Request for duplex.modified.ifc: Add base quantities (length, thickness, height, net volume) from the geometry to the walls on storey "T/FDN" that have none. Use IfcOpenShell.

First a look at what the model holds.

```python
import ifcopenshell
import ifcopenshell.util.element
import ifcopenshell.util.unit

model = ifcopenshell.open("duplex.modified.ifc")
print(model.schema)
for unit_type in ("LENGTHUNIT", "AREAUNIT", "VOLUMEUNIT"):
    print(unit_type, ifcopenshell.util.unit.calculate_unit_scale(model, unit_type))
storey = next(s for s in model.by_type("IfcBuildingStorey") if s.Name == "T/FDN")
walls = [e for e in ifcopenshell.util.element.get_decomposition(storey) if e.is_a("IfcWall")]
for e in sorted(walls, key=lambda e: e.id()):
    print(e.id(), e.is_a(), e.Name, list(ifcopenshell.util.element.get_psets(e, qtos_only=True)), sep=" | ")
```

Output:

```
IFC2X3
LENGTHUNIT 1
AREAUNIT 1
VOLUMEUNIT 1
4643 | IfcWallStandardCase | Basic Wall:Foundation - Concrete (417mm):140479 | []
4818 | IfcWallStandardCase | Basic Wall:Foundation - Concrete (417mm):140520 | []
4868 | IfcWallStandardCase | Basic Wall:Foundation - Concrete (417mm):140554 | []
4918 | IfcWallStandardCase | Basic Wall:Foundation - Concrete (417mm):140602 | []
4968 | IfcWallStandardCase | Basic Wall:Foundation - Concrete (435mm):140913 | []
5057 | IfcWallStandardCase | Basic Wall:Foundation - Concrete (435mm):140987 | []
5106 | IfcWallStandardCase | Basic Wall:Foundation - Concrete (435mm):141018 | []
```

```python
import ifcopenshell
import ifcopenshell.api.pset
import ifcopenshell.geom
import ifcopenshell.util.element
import ifcopenshell.util.shape
import ifcopenshell.util.unit

model = ifcopenshell.open("duplex.modified.ifc")
unit_scale = ifcopenshell.util.unit.calculate_unit_scale(model)
volume_scale = ifcopenshell.util.unit.calculate_unit_scale(model, "VOLUMEUNIT")
settings = ifcopenshell.geom.settings()

storey = next(s for s in model.by_type("IfcBuildingStorey") if s.Name == "T/FDN")
walls = [e for e in ifcopenshell.util.element.get_decomposition(storey) if e.is_a("IfcWall")]

for e in sorted(walls, key=lambda e: e.id()):
    if ifcopenshell.util.element.get_psets(e, qtos_only=True, should_inherit=False):
        continue
    # Geometry comes back in metres, in the element's own axes.
    shape = ifcopenshell.geom.create_shape(settings, e)
    values = {
        "Length": ifcopenshell.util.shape.get_x(shape.geometry) / unit_scale,
        "Width": ifcopenshell.util.shape.get_y(shape.geometry) / unit_scale,
        "Height": ifcopenshell.util.shape.get_z(shape.geometry) / unit_scale,
        "NetVolume": ifcopenshell.util.shape.get_volume(shape.geometry) / volume_scale,
    }
    qto = ifcopenshell.api.pset.add_qto(model, product=e, name="BaseQuantities")
    ifcopenshell.api.pset.edit_qto(model, qto=qto, properties=values)
    print(e.id(), {k: round(v, 3) for k, v in values.items()})

model.write("duplex.modified_updated.ifc")
```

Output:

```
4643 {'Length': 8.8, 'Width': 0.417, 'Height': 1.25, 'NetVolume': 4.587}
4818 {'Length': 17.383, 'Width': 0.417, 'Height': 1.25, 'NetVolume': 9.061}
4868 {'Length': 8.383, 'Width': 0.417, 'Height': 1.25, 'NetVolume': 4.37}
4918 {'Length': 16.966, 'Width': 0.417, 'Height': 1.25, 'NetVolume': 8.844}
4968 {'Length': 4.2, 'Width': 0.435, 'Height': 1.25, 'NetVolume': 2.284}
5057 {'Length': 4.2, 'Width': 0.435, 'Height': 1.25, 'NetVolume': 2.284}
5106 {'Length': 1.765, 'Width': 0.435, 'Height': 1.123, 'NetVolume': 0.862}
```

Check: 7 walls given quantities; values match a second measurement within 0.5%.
